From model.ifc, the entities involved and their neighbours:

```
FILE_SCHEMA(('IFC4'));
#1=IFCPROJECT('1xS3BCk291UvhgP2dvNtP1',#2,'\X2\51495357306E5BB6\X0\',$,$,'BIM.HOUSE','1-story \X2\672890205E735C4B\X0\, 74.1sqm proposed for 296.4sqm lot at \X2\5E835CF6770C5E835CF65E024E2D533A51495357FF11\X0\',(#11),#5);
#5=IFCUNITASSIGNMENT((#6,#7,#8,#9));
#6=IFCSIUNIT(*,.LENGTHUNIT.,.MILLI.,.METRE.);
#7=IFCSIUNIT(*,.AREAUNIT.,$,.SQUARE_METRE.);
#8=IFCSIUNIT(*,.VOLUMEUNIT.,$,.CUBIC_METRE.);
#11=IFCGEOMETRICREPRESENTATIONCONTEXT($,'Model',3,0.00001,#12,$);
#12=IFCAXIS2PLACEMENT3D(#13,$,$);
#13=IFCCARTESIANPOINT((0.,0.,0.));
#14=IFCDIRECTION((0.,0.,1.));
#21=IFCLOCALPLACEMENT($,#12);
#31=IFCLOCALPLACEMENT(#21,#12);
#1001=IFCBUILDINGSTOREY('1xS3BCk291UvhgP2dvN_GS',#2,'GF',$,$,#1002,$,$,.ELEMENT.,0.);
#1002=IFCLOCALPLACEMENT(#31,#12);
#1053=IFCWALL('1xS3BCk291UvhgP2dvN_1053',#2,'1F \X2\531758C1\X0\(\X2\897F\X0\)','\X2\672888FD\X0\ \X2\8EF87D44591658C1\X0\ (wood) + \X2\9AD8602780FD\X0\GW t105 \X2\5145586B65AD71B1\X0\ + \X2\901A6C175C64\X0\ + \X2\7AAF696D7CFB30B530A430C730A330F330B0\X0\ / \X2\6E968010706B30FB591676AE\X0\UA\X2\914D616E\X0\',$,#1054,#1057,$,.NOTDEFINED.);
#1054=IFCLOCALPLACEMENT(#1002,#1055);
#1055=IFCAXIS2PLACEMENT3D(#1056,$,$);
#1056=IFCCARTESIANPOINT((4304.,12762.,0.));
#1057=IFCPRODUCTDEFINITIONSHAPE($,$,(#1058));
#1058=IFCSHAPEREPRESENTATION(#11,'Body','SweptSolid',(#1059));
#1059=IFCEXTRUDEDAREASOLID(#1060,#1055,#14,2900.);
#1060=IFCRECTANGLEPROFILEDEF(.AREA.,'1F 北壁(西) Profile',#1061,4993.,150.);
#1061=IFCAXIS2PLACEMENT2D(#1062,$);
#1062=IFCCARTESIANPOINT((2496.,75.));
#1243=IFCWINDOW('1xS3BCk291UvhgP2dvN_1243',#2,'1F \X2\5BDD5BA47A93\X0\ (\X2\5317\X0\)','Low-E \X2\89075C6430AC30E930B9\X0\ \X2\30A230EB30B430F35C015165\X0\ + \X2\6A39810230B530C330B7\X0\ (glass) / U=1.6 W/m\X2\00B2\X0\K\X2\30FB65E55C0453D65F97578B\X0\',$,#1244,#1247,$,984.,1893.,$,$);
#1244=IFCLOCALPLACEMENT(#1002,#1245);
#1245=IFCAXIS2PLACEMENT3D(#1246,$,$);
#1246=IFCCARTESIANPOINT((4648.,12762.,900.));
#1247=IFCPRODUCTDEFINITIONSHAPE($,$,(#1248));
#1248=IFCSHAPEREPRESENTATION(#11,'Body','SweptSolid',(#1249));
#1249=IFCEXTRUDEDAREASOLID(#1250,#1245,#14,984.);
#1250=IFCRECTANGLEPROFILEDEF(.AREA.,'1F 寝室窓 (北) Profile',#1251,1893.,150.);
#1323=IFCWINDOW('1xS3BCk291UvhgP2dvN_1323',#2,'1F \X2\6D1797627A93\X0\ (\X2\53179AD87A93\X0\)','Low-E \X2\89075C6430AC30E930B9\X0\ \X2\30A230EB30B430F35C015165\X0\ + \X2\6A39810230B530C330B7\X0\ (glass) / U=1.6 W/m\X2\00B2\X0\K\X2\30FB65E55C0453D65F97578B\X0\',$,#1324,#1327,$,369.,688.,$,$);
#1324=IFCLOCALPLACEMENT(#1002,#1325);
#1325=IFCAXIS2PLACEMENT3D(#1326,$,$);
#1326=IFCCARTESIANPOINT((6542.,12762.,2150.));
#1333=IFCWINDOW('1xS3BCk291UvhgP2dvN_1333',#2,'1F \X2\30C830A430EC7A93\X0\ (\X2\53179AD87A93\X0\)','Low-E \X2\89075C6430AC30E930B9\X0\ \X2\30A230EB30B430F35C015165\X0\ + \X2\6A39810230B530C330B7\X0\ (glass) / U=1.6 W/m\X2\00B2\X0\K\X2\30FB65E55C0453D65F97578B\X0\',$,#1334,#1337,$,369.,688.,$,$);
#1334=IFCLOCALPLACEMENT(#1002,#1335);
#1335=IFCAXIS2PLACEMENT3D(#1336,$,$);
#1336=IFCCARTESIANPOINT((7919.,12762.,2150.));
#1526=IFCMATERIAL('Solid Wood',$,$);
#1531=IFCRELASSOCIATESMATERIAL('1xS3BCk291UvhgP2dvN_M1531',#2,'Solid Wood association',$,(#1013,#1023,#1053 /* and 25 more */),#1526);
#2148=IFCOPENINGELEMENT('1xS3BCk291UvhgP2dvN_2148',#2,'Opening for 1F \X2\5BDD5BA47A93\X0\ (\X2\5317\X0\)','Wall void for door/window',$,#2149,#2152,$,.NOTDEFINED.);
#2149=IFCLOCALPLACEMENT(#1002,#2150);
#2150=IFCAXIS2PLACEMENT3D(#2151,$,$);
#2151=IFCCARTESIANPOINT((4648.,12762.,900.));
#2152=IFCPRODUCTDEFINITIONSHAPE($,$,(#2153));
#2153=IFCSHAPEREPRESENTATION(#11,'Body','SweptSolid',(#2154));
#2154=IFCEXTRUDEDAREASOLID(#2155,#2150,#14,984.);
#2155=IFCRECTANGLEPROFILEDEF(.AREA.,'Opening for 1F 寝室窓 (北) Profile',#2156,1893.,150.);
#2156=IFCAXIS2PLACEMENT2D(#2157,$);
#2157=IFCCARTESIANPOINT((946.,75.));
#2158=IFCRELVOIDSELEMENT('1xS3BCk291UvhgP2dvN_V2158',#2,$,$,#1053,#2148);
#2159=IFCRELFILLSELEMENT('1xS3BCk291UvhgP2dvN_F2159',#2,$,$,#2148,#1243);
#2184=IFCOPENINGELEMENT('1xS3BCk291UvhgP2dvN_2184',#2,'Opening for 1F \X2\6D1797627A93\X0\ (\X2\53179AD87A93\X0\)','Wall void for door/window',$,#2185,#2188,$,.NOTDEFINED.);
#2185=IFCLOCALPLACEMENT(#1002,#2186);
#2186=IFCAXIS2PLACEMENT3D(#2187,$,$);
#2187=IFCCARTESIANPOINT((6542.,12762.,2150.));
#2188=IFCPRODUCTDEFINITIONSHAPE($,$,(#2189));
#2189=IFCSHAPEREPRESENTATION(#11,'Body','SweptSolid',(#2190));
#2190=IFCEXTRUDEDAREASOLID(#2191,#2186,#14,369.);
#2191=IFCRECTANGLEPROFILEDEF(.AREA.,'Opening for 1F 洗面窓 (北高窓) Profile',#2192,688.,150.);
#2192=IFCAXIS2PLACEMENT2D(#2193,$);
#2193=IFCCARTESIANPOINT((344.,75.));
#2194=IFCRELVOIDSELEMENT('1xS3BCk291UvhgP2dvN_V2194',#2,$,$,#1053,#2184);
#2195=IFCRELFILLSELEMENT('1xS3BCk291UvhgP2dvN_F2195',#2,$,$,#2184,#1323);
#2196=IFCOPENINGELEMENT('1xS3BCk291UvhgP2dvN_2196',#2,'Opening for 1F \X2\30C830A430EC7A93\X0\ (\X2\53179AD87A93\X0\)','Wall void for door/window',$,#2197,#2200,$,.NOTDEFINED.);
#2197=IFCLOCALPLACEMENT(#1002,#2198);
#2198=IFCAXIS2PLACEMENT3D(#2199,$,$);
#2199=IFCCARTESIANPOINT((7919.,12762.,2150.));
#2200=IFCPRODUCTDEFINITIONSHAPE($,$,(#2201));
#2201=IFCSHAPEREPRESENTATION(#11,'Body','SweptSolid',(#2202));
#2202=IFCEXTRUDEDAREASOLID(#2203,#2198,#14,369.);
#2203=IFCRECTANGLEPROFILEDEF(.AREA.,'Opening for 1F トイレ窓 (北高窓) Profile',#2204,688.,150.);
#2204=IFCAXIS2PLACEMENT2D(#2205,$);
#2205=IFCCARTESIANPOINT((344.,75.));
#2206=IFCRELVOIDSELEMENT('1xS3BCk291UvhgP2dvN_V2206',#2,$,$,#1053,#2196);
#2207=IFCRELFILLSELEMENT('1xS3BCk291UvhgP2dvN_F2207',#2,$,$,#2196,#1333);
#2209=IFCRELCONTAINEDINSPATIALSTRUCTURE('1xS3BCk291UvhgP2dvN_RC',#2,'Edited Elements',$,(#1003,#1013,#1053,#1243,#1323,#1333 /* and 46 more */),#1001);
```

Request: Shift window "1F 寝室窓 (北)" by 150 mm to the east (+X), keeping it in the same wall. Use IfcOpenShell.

```python
import ifcopenshell
import ifcopenshell.api.geometry
import ifcopenshell.util.placement

model = ifcopenshell.open("model.ifc")

window = model.by_guid("1xS3BCk291UvhgP2dvN_1243")
opening = window.FillsVoids[0].RelatingOpeningElement
wall = opening.VoidsElements[0].RelatingBuildingElement

wall_matrix = ifcopenshell.util.placement.get_local_placement(wall.ObjectPlacement)
shift = wall_matrix[:3, 0] * 150.0
before = ifcopenshell.util.placement.get_local_placement(window.ObjectPlacement)[:3, 3].copy()

# The window is not placed relative to its opening, so move both.
for product in (opening, window):
    matrix = ifcopenshell.util.placement.get_local_placement(product.ObjectPlacement)
    matrix[:3, 3] += shift
    ifcopenshell.api.geometry.edit_object_placement(model, product=product, matrix=matrix, is_si=False)

after = ifcopenshell.util.placement.get_local_placement(window.ObjectPlacement)[:3, 3]
print("window moved by", (after - before).round(3) + 0.0)

model.write("model_v2.ifc")
```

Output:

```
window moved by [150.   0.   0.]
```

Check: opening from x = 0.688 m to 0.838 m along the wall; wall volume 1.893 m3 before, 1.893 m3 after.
